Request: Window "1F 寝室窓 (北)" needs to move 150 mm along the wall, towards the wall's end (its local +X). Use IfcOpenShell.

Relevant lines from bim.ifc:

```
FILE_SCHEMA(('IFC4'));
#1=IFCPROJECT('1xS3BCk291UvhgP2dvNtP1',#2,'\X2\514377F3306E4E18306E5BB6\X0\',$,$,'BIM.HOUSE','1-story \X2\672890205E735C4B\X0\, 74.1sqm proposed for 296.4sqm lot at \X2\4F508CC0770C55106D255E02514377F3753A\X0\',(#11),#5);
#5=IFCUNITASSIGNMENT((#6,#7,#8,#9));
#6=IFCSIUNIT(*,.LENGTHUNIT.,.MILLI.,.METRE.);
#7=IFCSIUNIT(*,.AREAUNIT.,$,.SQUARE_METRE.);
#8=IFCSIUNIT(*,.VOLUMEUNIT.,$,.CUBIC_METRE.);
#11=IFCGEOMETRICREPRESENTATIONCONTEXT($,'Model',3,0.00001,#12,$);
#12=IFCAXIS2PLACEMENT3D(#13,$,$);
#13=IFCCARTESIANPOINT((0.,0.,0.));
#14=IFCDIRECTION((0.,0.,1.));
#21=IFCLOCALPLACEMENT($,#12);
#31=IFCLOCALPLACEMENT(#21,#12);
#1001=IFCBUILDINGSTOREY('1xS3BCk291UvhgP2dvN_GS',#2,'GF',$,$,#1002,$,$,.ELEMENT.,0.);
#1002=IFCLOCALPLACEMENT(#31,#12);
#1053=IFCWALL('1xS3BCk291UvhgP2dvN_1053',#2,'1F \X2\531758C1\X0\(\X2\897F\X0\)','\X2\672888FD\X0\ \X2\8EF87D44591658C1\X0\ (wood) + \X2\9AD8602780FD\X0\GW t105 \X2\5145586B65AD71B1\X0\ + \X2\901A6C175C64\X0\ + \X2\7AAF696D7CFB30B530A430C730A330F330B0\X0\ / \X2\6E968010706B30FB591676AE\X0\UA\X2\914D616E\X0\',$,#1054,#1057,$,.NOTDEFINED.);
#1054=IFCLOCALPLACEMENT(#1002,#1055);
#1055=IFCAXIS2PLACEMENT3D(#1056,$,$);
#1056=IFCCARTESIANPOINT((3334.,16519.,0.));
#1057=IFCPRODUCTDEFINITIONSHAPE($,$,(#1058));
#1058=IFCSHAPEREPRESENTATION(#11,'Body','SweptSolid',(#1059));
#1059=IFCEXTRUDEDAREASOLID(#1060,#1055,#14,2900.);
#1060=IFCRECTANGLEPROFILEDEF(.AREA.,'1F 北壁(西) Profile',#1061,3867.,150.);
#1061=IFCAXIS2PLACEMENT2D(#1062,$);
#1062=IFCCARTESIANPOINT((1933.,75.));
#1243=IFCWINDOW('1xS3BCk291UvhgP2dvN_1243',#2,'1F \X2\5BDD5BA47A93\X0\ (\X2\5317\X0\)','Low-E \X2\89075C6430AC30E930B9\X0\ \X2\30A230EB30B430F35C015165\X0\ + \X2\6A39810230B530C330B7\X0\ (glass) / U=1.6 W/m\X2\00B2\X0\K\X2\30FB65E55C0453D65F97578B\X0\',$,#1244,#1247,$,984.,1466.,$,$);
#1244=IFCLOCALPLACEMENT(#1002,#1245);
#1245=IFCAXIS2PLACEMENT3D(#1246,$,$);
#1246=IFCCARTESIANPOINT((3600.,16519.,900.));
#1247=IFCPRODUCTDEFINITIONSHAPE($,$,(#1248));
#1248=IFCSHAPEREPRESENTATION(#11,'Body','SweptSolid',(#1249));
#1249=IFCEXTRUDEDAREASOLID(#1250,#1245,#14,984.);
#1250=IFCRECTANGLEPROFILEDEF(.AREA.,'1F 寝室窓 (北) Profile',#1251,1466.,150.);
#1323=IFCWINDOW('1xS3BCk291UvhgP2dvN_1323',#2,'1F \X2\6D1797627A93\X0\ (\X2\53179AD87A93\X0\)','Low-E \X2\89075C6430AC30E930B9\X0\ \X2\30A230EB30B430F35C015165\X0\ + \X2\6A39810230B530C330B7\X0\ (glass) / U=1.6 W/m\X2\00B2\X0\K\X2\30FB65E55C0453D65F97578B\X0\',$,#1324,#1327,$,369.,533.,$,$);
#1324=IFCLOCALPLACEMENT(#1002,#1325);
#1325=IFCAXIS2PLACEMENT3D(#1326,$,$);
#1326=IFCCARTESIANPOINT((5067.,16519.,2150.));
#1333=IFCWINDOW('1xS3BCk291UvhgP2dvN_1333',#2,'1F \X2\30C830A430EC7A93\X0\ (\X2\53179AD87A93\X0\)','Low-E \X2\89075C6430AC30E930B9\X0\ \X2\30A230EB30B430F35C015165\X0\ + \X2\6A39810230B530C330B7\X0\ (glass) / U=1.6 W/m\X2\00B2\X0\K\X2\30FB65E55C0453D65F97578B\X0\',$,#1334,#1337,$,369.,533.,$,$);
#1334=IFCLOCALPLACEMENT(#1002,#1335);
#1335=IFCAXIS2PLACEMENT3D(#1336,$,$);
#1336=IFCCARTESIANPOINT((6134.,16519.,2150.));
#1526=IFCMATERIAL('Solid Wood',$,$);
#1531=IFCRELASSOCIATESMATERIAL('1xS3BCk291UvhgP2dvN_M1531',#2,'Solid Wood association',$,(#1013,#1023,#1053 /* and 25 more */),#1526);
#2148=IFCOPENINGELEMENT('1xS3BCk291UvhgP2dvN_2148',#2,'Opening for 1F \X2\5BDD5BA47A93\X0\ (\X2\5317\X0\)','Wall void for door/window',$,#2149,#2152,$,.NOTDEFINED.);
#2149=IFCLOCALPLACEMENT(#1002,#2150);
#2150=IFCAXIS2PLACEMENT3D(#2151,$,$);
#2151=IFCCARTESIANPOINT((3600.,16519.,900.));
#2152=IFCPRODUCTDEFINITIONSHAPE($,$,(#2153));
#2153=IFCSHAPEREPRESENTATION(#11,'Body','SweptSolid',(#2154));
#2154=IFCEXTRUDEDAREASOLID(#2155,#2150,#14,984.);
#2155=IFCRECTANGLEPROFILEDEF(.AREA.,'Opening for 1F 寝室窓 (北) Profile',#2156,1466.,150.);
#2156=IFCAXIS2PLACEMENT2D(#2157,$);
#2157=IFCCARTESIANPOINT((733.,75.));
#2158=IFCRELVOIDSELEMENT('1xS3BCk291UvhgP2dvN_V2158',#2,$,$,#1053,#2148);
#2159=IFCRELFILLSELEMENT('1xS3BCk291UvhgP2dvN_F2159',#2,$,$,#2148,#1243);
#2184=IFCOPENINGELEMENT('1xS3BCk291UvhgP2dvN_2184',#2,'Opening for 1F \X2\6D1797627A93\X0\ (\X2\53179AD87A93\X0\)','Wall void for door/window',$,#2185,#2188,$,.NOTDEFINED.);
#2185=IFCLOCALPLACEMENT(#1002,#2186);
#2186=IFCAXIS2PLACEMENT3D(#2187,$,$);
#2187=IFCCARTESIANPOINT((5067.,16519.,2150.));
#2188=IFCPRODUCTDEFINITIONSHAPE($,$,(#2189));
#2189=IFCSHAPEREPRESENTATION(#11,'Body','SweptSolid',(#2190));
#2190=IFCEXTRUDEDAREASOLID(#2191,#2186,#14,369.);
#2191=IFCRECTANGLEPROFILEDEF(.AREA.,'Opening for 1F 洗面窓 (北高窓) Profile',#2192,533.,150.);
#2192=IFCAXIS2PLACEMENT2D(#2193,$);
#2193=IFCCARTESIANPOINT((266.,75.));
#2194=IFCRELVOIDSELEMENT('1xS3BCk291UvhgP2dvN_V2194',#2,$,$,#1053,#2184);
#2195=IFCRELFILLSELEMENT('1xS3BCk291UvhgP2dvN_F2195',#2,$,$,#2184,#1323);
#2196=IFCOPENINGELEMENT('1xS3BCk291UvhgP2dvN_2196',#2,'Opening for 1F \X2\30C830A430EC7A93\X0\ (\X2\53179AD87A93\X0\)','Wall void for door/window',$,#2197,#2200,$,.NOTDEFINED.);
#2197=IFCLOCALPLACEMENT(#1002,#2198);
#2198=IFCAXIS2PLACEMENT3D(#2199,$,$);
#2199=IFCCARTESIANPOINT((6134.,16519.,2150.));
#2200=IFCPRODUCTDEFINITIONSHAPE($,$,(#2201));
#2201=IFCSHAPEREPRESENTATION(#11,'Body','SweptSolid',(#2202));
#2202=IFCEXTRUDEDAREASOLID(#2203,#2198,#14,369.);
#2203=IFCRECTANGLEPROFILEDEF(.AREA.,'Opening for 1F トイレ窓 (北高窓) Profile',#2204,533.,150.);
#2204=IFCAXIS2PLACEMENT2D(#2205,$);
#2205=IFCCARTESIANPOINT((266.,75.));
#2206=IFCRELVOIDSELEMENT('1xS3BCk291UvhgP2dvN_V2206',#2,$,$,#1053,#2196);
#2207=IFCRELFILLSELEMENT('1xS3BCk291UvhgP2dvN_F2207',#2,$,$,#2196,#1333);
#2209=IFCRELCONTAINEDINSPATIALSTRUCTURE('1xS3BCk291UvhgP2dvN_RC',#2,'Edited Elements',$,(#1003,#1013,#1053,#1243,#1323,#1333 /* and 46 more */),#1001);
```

```python
import ifcopenshell
import ifcopenshell.api.geometry
import ifcopenshell.util.placement

model = ifcopenshell.open("bim.ifc")

window = model.by_id(1243)
opening = window.FillsVoids[0].RelatingOpeningElement
wall = opening.VoidsElements[0].RelatingBuildingElement

wall_matrix = ifcopenshell.util.placement.get_local_placement(wall.ObjectPlacement)
shift = wall_matrix[:3, 0] * 150.0
before = ifcopenshell.util.placement.get_local_placement(window.ObjectPlacement)[:3, 3].copy()

# The window is not placed relative to its opening, so move both.
for product in (opening, window):
    matrix = ifcopenshell.util.placement.get_local_placement(product.ObjectPlacement)
    matrix[:3, 3] += shift
    ifcopenshell.api.geometry.edit_object_placement(model, product=product, matrix=matrix, is_si=False)

after = ifcopenshell.util.placement.get_local_placement(window.ObjectPlacement)[:3, 3]
print("window moved by", (after - before).round(3) + 0.0)

model.write("bim_edited.ifc")
```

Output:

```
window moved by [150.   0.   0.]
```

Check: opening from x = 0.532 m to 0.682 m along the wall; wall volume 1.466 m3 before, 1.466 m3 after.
